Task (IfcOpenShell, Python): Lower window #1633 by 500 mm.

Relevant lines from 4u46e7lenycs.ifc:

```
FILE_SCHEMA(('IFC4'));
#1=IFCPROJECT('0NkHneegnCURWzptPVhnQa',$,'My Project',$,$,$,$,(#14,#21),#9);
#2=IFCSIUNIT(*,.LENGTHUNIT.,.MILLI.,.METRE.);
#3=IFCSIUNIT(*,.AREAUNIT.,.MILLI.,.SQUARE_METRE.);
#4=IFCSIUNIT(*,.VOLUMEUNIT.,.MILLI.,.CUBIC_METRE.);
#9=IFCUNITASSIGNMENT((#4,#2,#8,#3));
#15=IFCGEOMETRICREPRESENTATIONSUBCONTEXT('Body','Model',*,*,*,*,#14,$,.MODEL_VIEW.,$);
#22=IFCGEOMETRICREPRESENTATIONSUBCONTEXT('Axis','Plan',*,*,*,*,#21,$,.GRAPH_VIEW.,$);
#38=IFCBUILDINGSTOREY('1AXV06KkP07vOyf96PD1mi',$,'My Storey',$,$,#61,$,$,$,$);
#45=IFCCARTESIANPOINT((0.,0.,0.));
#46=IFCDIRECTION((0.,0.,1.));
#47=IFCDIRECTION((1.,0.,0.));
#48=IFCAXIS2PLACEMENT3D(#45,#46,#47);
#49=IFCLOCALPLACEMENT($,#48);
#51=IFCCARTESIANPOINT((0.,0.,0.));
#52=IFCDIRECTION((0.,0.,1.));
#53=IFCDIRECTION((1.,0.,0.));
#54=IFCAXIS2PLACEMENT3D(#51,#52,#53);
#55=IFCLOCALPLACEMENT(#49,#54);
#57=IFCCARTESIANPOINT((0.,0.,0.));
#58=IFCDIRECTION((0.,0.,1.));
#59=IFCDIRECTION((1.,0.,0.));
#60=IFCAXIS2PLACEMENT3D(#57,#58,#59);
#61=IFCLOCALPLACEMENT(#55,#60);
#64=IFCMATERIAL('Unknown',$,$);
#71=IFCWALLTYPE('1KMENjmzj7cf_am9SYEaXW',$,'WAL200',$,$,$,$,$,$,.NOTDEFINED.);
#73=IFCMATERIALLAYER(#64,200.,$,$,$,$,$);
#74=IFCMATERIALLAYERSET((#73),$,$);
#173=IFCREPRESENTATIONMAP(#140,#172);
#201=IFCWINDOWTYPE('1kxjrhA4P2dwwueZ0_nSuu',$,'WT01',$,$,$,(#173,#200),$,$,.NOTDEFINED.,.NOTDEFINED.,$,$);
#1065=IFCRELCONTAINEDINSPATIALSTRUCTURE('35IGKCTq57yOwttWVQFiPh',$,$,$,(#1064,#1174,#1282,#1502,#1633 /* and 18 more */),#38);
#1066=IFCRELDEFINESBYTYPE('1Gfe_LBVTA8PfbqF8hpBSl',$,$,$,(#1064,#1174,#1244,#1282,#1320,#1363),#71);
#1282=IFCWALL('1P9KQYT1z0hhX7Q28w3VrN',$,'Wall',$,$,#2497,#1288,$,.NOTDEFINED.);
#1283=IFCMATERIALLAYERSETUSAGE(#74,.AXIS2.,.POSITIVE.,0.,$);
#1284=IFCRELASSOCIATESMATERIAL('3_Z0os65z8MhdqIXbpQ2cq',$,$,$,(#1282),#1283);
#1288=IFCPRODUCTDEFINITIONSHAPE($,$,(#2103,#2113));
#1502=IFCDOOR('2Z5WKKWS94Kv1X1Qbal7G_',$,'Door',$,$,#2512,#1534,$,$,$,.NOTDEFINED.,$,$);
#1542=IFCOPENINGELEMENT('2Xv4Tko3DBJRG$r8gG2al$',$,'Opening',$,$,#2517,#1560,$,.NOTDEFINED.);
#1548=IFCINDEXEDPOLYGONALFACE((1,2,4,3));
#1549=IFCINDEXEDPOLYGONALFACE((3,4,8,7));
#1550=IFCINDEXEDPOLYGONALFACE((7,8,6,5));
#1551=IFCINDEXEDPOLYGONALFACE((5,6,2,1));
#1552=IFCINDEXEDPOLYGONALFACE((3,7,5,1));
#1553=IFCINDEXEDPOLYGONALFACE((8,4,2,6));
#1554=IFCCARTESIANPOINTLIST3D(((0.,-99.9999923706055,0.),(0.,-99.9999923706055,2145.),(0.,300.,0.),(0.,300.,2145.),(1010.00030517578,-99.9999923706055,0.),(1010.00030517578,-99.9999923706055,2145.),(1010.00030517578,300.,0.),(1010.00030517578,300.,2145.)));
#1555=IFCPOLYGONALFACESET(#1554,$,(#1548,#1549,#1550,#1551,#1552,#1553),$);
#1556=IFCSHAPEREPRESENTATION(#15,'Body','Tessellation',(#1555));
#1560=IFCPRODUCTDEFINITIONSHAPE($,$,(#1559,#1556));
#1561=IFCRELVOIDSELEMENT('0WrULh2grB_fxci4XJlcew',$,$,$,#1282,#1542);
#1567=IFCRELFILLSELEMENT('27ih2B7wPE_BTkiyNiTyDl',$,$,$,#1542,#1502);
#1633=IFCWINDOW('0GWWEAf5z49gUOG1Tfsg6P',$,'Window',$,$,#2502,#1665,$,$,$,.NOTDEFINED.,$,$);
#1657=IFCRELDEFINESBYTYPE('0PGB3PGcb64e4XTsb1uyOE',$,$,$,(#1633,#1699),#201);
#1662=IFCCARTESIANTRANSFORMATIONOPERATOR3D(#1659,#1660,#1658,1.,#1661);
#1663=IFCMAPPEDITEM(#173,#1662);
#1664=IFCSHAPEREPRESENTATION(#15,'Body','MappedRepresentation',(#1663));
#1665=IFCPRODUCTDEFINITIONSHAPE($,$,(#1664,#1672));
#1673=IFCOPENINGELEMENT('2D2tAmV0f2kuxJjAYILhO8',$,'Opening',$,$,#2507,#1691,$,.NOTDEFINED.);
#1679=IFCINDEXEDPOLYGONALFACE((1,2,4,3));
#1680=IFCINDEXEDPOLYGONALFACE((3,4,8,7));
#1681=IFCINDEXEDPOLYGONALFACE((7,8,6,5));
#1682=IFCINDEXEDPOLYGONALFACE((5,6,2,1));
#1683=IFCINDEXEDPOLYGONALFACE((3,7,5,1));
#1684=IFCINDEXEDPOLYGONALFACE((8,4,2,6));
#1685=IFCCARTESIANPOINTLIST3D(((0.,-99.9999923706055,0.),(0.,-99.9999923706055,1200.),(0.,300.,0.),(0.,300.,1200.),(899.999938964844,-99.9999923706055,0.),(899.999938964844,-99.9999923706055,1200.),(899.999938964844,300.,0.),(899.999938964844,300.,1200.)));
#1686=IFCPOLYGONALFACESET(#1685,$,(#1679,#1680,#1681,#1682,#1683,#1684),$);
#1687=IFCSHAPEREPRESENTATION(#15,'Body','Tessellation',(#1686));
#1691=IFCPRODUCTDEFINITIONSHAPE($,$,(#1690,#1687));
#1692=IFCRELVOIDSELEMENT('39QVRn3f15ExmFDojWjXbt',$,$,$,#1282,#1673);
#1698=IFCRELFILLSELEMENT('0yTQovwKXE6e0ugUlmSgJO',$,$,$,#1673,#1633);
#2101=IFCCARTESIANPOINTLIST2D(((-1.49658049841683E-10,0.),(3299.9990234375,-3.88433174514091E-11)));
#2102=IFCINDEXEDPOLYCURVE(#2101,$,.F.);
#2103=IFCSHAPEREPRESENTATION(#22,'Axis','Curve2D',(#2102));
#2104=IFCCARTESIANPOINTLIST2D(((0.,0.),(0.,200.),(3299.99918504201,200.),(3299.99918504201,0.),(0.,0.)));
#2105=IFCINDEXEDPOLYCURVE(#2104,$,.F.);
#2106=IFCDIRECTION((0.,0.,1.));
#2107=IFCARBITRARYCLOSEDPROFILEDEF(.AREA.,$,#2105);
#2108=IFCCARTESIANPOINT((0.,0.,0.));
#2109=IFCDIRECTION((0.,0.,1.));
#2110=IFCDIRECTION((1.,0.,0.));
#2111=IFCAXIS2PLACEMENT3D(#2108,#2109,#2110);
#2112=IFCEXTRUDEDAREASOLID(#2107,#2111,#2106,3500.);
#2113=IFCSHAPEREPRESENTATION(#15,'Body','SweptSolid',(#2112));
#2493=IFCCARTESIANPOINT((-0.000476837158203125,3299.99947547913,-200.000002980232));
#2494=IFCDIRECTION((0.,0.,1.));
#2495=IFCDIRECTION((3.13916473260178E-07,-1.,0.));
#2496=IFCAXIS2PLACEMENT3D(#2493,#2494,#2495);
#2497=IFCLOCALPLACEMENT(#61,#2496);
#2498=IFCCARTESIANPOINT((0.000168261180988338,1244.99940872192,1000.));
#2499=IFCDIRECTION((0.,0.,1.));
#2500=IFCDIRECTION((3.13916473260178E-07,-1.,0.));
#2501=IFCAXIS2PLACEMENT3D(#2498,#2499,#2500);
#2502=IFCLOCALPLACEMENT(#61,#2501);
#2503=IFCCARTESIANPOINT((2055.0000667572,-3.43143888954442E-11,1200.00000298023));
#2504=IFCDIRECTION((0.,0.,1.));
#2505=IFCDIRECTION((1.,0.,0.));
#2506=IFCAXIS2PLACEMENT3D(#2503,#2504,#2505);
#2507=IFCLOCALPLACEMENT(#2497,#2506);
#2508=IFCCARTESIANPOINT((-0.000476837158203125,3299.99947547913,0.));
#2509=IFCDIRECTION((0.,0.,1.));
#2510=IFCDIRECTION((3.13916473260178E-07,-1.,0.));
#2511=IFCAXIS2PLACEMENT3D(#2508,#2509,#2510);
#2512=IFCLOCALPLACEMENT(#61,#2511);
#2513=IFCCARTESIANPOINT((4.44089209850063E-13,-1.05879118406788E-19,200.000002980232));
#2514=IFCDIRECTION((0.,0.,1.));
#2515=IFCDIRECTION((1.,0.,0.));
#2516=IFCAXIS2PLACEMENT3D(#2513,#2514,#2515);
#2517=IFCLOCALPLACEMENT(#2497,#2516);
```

```python
import numpy as np
import ifcopenshell
import ifcopenshell.api.geometry
import ifcopenshell.util.placement
import ifcopenshell.util.unit

model = ifcopenshell.open("4u46e7lenycs.ifc")
unit_scale = ifcopenshell.util.unit.calculate_unit_scale(model)

window = model.by_id(1633)
opening = window.FillsVoids[0].RelatingOpeningElement
dz = -0.5 / unit_scale

shift = np.array([0.0, 0.0, dz])
# The window is not placed relative to its opening, so move both.
for product in (opening, window):
    matrix = ifcopenshell.util.placement.get_local_placement(product.ObjectPlacement)
    matrix[:3, 3] += shift
    ifcopenshell.api.geometry.edit_object_placement(model, product=product, matrix=matrix, is_si=False)

print(f"moved by {dz * unit_scale:+.3f} m")

model.write("4u46e7lenycs_rev.ifc")
```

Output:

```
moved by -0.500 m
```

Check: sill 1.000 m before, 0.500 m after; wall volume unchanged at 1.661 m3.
